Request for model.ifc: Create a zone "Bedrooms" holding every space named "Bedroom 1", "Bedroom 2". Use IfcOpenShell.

First a look at what the model holds.

```python
import ifcopenshell

model = ifcopenshell.open("model.ifc")
print(model.schema)
seen = {}
for space in model.by_type("IfcSpace"):
    seen[space.LongName] = seen.get(space.LongName, 0) + 1
for name, count in sorted(seen.items(), key=str):
    print(count, "x", name)
print("zones:", [z.Name for z in model.by_type("IfcZone")][:20])
```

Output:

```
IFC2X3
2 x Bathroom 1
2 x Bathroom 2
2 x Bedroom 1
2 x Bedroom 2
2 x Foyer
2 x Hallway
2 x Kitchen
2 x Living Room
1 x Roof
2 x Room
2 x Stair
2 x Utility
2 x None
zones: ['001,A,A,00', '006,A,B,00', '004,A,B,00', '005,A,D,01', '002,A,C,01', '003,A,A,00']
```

```python
import ifcopenshell
import ifcopenshell.api.group
import ifcopenshell.api.root

model = ifcopenshell.open("model.ifc")

names = {"Bedroom 1", "Bedroom 2"}
spaces = [s for s in model.by_type("IfcSpace") if s.LongName in names]

zone = ifcopenshell.api.root.create_entity(model, ifc_class="IfcZone", name="Bedrooms")
ifcopenshell.api.group.assign_group(model, products=spaces, group=zone)
print(len(spaces), "spaces in", zone.Name)

model.write("model_updated.ifc")
```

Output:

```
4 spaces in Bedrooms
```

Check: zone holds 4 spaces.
